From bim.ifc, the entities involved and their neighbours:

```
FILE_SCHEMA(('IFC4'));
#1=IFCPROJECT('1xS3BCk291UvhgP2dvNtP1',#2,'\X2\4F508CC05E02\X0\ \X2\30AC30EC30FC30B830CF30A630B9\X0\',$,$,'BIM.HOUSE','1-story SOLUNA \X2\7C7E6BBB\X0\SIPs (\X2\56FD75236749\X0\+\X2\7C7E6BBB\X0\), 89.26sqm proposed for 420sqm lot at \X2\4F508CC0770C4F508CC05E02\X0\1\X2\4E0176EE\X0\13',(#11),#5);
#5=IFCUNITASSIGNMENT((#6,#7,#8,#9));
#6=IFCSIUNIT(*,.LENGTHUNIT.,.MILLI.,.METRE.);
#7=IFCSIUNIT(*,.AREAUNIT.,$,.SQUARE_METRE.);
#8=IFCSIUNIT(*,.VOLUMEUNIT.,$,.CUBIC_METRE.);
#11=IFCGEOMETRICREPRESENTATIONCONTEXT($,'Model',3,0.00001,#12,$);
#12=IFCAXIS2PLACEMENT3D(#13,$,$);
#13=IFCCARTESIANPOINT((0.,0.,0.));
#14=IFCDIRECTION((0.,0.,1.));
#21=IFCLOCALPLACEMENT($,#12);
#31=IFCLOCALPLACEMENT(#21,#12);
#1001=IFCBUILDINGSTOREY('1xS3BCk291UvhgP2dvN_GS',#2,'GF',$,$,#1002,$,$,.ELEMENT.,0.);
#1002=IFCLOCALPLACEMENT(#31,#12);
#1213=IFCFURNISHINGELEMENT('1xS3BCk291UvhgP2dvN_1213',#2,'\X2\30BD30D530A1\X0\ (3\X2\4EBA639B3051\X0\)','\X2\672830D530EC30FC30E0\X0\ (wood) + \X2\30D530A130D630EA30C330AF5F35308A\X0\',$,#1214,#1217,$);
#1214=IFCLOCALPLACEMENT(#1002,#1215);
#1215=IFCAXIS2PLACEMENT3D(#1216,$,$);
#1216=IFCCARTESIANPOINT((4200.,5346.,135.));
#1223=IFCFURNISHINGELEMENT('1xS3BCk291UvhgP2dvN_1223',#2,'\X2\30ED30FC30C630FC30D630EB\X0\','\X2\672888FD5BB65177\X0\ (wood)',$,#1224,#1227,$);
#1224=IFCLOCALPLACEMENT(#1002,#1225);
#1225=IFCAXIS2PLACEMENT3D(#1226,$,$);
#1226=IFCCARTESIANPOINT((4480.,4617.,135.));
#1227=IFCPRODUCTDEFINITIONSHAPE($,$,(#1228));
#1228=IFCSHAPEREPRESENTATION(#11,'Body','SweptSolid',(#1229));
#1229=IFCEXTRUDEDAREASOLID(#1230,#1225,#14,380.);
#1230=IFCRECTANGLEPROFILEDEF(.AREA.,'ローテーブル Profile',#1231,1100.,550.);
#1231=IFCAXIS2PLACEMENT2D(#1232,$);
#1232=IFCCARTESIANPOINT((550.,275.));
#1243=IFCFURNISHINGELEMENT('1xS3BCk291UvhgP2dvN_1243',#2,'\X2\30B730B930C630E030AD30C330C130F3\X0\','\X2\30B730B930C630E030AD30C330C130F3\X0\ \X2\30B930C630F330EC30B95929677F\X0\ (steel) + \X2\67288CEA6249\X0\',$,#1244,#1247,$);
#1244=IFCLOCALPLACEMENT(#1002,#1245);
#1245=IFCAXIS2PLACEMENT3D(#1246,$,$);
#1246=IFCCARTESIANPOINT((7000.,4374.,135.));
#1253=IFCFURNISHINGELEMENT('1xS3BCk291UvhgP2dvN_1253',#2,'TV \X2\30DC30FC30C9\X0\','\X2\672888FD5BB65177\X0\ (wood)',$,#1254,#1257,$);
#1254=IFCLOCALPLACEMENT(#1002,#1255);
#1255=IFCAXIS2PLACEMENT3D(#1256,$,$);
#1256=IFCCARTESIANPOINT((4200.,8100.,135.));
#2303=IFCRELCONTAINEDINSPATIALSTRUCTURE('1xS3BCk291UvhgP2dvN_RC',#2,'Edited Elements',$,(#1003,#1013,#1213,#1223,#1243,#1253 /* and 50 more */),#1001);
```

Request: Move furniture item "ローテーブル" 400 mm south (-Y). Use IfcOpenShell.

```python
import ifcopenshell
import ifcopenshell.api.geometry
import ifcopenshell.util.placement

model = ifcopenshell.open("bim.ifc")

item = model.by_guid("1xS3BCk291UvhgP2dvN_1223")
matrix = ifcopenshell.util.placement.get_local_placement(item.ObjectPlacement)
matrix[1, 3] -= 400.0
ifcopenshell.api.geometry.edit_object_placement(model, product=item, matrix=matrix, is_si=False)

print(ifcopenshell.util.placement.get_local_placement(item.ObjectPlacement).round(3) + 0.0)

model.write("bim_rev.ifc")
```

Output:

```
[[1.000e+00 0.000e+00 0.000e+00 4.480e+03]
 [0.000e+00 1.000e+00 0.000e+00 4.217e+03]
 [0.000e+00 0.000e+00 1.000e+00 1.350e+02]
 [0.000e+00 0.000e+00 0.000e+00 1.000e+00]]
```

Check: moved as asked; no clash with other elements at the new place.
